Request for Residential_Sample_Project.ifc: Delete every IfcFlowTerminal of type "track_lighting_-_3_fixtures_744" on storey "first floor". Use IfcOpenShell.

First a look at what the model holds.

```python
import ifcopenshell
import ifcopenshell.util.element

model = ifcopenshell.open("Residential_Sample_Project.ifc")
print(model.schema)
storey = next(s for s in model.by_type("IfcBuildingStorey") if s.Name == "first floor")
terminals = [e for e in ifcopenshell.util.element.get_decomposition(storey) if e.is_a("IfcFlowTerminal")]
seen = {}
for e in terminals:
    element_type = ifcopenshell.util.element.get_type(e)
    name = element_type.Name if element_type not in (None, e) else None
    seen[name] = seen.get(name, 0) + 1
for name, count in sorted(seen.items(), key=str):
    print(count, "x", name)
```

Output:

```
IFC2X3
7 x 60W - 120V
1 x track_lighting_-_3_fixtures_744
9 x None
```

```python
import ifcopenshell
import ifcopenshell.api.root
import ifcopenshell.util.element

model = ifcopenshell.open("Residential_Sample_Project.ifc")

storey = next(s for s in model.by_type("IfcBuildingStorey") if s.Name == "first floor")
terminals = [e for e in ifcopenshell.util.element.get_decomposition(storey) if e.is_a("IfcFlowTerminal")]
targets = [e for e in terminals if (t := ifcopenshell.util.element.get_type(e)) not in (None, e) and t.Name == "track_lighting_-_3_fixtures_744"]

for e in targets:
    ifcopenshell.api.root.remove_product(model, product=e)
print(len(targets), "removed")

model.write("Residential_Sample_Project_rev.ifc")
```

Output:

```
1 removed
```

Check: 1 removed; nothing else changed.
